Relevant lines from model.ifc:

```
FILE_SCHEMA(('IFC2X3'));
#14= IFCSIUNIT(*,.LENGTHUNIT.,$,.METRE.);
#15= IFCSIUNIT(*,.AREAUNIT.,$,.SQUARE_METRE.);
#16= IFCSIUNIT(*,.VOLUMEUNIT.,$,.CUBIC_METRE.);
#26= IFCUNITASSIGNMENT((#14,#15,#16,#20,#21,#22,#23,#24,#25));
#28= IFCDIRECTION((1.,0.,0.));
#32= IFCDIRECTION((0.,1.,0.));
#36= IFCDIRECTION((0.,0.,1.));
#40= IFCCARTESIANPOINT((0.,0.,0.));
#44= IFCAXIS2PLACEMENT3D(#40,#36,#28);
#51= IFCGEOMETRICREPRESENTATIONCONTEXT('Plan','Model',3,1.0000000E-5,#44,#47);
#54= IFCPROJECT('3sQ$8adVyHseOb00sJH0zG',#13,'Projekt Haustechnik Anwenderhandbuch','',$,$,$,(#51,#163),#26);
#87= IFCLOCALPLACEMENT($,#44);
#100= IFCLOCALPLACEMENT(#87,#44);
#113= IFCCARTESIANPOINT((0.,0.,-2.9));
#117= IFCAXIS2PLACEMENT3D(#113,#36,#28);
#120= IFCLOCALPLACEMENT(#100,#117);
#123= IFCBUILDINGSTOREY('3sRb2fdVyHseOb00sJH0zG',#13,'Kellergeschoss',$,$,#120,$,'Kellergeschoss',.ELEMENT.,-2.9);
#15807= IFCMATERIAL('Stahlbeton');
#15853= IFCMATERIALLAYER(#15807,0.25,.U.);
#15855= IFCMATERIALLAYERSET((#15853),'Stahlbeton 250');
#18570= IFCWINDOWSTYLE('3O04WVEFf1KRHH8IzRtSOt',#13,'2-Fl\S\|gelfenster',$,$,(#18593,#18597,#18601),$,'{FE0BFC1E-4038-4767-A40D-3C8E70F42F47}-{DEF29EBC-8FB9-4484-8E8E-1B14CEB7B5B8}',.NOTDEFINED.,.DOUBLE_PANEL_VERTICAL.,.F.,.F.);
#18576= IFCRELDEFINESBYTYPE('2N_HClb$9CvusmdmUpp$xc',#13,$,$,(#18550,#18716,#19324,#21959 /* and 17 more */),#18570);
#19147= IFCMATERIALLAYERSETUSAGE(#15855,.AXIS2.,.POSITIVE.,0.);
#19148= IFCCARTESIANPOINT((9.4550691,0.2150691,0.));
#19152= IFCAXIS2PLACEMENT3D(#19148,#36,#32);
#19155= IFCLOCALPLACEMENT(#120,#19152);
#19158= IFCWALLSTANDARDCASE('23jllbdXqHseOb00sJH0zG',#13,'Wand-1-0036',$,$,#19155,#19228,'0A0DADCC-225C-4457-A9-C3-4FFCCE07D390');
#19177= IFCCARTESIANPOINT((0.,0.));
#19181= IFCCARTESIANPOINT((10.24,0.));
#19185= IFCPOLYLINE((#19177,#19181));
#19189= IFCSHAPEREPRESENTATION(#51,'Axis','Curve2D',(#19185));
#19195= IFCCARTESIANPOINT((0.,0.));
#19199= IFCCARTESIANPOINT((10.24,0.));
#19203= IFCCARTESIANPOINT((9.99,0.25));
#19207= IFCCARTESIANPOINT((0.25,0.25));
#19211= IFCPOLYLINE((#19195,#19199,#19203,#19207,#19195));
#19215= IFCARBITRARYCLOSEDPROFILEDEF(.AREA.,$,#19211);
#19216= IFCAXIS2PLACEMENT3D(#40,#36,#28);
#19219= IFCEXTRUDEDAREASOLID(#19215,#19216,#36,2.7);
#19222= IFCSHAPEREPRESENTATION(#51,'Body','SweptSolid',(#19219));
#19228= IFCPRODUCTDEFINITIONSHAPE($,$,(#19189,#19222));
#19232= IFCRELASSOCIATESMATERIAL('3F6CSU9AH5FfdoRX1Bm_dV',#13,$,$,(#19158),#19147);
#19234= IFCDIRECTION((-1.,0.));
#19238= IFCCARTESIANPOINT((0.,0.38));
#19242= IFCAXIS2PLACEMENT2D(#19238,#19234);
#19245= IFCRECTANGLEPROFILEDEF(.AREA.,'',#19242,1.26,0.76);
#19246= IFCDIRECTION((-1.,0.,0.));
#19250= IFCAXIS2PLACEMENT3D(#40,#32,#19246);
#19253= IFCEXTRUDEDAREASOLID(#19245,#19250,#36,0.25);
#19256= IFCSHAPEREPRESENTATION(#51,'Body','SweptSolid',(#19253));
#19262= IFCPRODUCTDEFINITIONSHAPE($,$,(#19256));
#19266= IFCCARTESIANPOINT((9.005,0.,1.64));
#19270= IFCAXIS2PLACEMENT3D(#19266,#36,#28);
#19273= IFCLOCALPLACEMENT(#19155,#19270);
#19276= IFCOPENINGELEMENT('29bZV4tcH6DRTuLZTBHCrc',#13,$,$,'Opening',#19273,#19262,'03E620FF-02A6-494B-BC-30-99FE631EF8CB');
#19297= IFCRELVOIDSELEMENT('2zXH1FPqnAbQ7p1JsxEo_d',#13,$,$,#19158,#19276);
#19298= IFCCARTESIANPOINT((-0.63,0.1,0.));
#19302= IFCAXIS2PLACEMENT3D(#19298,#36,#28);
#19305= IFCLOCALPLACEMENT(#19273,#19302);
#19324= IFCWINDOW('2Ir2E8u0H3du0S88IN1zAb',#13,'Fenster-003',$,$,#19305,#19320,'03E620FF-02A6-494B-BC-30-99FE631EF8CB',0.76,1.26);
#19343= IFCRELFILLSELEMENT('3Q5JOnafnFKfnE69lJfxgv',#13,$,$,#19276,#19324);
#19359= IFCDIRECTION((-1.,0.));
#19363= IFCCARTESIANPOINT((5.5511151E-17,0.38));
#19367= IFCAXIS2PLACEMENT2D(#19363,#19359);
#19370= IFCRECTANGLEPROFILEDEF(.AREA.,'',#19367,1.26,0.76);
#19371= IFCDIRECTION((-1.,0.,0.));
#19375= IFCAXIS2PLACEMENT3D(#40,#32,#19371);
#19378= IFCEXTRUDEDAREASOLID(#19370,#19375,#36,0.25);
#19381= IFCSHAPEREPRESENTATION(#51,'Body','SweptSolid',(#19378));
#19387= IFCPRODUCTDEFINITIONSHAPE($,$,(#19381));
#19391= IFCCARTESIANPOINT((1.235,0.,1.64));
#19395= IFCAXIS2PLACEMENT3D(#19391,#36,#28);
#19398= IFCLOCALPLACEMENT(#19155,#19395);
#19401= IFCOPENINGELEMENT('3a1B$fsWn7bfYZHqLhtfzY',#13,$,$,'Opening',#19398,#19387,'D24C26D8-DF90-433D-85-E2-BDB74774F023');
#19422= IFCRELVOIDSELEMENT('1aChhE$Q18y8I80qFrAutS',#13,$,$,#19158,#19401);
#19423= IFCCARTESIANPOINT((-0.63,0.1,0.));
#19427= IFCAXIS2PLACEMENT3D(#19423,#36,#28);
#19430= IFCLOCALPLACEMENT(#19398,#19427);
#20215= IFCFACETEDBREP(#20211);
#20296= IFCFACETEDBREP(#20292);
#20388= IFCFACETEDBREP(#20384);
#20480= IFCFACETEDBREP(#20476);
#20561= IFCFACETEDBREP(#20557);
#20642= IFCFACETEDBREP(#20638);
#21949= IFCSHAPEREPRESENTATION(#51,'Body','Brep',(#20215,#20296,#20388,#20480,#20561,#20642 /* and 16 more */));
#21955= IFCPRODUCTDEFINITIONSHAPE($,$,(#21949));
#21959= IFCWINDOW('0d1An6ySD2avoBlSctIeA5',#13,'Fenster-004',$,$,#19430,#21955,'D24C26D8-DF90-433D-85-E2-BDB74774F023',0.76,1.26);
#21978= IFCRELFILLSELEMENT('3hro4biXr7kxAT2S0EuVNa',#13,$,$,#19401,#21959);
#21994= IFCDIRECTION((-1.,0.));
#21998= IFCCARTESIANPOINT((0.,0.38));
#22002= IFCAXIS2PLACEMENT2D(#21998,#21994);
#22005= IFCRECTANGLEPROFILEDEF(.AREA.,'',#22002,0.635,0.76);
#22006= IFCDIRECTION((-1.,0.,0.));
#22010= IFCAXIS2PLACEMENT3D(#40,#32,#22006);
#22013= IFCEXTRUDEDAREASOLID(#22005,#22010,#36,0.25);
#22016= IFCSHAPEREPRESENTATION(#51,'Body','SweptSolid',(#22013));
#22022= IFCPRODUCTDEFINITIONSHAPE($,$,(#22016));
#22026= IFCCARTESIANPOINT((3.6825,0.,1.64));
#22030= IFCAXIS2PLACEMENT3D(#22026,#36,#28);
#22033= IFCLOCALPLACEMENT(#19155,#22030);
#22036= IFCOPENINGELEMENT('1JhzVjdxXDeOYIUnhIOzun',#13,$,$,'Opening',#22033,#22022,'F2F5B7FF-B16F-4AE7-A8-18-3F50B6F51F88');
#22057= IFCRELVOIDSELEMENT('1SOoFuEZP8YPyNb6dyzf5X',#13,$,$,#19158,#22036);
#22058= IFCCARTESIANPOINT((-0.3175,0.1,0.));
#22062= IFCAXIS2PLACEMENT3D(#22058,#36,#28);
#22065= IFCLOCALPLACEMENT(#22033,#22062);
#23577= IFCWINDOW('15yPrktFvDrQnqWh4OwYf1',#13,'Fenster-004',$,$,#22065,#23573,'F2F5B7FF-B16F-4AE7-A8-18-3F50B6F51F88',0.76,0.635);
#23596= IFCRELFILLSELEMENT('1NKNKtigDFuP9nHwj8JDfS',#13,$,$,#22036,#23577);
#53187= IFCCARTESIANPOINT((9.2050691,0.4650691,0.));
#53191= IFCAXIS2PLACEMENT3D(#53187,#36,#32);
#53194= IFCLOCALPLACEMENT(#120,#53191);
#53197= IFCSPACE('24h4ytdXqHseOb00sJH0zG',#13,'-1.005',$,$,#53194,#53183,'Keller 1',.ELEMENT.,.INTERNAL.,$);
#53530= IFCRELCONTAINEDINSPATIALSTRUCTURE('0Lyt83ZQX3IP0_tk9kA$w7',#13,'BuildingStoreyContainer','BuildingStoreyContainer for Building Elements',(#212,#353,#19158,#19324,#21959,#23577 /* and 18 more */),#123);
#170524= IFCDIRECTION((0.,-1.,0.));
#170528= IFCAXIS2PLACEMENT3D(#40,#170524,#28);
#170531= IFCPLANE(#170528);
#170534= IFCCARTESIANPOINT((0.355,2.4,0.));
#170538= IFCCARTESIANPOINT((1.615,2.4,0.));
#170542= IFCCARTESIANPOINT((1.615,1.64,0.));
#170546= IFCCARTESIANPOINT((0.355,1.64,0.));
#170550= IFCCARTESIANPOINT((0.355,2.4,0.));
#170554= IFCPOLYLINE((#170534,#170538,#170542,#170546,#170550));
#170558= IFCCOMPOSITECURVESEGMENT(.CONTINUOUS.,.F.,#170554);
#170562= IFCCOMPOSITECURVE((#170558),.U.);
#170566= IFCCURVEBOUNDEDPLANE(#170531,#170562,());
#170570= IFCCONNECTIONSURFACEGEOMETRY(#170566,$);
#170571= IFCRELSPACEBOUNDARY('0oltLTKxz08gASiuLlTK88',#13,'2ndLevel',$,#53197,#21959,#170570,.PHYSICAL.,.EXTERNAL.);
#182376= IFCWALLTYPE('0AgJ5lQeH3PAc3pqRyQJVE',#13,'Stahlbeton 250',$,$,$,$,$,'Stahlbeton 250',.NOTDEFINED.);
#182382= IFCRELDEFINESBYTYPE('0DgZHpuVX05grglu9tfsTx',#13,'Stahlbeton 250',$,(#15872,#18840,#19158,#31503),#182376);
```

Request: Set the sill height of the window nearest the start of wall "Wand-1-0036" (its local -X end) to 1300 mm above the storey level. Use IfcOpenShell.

```python
import numpy as np
import ifcopenshell
import ifcopenshell.api.geometry
import ifcopenshell.geom
import ifcopenshell.util.element
import ifcopenshell.util.placement
import ifcopenshell.util.shape
import ifcopenshell.util.unit

model = ifcopenshell.open("model.ifc")
unit_scale = ifcopenshell.util.unit.calculate_unit_scale(model)

window = model.by_guid("0d1An6ySD2avoBlSctIeA5")
opening = window.FillsVoids[0].RelatingOpeningElement
storey = ifcopenshell.util.element.get_container(window, ifc_class="IfcBuildingStorey")
level = ifcopenshell.util.placement.get_local_placement(storey.ObjectPlacement)[2, 3]

# The opening's origin need not be at the sill, so measure its lowest point.
shape = ifcopenshell.geom.create_shape(ifcopenshell.geom.settings(), opening)
bottom = ifcopenshell.util.shape.get_shape_bottom_elevation(shape, shape.geometry) / unit_scale
dz = level + 1.3 - bottom

shift = np.array([0.0, 0.0, dz])
# The window is placed relative to its opening, so it follows when the opening moves.
matrix = ifcopenshell.util.placement.get_local_placement(opening.ObjectPlacement)
matrix[:3, 3] += shift
ifcopenshell.api.geometry.edit_object_placement(
    model, product=opening, matrix=matrix, is_si=False, should_transform_children=True
)

# Space boundary surfaces are stored in each space's coordinates; move them too.
for rel in window.ProvidesBoundaries:
    if not rel.ConnectionGeometry:
        continue
    surface = rel.ConnectionGeometry.SurfaceOnRelatingElement.BasisSurface
    space_matrix = ifcopenshell.util.placement.get_local_placement(rel.RelatingSpace.ObjectPlacement)
    point = np.array(surface.Position.Location.Coordinates) + space_matrix[:3, :3].T @ shift
    surface.Position = model.createIfcAxis2Placement3D(
        model.createIfcCartesianPoint(point.tolist()), surface.Position.Axis, surface.Position.RefDirection
    )

print(f"moved by {dz * unit_scale:+.3f} m")

model.write("model_edited.ifc")
```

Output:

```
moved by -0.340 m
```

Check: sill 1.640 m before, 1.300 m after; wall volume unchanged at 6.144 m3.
